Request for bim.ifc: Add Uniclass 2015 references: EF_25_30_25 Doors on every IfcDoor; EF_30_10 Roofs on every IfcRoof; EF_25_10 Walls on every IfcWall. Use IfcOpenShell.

First a look at what the model holds.

```python
import ifcopenshell

model = ifcopenshell.open("bim.ifc")
print(model.schema)
print("classifications:", [c.Name for c in model.by_type("IfcClassification")])
for ifc_class in ("IfcDoor", "IfcRoof", "IfcStair", "IfcWall", "IfcWindow"):
    print(ifc_class, len(model.by_type(ifc_class)))
```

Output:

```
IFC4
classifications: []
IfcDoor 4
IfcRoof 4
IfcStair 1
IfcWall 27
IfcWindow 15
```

```python
import ifcopenshell
import ifcopenshell.api.classification

model = ifcopenshell.open("bim.ifc")

system = ifcopenshell.api.classification.add_classification(model, classification="Uniclass 2015")

codes = {
    "IfcDoor": ("EF_25_30_25", "Doors"),
    "IfcRoof": ("EF_30_10", "Roofs"),
    "IfcWall": ("EF_25_10", "Walls"),
}
for ifc_class, (code, name) in codes.items():
    products = model.by_type(ifc_class)
    ifcopenshell.api.classification.add_reference(
        model, products=products, classification=system, identification=code, name=name
    )
    print(code, len(products))

model.write("bim_rev.ifc")
```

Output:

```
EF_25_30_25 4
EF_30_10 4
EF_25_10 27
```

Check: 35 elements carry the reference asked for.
